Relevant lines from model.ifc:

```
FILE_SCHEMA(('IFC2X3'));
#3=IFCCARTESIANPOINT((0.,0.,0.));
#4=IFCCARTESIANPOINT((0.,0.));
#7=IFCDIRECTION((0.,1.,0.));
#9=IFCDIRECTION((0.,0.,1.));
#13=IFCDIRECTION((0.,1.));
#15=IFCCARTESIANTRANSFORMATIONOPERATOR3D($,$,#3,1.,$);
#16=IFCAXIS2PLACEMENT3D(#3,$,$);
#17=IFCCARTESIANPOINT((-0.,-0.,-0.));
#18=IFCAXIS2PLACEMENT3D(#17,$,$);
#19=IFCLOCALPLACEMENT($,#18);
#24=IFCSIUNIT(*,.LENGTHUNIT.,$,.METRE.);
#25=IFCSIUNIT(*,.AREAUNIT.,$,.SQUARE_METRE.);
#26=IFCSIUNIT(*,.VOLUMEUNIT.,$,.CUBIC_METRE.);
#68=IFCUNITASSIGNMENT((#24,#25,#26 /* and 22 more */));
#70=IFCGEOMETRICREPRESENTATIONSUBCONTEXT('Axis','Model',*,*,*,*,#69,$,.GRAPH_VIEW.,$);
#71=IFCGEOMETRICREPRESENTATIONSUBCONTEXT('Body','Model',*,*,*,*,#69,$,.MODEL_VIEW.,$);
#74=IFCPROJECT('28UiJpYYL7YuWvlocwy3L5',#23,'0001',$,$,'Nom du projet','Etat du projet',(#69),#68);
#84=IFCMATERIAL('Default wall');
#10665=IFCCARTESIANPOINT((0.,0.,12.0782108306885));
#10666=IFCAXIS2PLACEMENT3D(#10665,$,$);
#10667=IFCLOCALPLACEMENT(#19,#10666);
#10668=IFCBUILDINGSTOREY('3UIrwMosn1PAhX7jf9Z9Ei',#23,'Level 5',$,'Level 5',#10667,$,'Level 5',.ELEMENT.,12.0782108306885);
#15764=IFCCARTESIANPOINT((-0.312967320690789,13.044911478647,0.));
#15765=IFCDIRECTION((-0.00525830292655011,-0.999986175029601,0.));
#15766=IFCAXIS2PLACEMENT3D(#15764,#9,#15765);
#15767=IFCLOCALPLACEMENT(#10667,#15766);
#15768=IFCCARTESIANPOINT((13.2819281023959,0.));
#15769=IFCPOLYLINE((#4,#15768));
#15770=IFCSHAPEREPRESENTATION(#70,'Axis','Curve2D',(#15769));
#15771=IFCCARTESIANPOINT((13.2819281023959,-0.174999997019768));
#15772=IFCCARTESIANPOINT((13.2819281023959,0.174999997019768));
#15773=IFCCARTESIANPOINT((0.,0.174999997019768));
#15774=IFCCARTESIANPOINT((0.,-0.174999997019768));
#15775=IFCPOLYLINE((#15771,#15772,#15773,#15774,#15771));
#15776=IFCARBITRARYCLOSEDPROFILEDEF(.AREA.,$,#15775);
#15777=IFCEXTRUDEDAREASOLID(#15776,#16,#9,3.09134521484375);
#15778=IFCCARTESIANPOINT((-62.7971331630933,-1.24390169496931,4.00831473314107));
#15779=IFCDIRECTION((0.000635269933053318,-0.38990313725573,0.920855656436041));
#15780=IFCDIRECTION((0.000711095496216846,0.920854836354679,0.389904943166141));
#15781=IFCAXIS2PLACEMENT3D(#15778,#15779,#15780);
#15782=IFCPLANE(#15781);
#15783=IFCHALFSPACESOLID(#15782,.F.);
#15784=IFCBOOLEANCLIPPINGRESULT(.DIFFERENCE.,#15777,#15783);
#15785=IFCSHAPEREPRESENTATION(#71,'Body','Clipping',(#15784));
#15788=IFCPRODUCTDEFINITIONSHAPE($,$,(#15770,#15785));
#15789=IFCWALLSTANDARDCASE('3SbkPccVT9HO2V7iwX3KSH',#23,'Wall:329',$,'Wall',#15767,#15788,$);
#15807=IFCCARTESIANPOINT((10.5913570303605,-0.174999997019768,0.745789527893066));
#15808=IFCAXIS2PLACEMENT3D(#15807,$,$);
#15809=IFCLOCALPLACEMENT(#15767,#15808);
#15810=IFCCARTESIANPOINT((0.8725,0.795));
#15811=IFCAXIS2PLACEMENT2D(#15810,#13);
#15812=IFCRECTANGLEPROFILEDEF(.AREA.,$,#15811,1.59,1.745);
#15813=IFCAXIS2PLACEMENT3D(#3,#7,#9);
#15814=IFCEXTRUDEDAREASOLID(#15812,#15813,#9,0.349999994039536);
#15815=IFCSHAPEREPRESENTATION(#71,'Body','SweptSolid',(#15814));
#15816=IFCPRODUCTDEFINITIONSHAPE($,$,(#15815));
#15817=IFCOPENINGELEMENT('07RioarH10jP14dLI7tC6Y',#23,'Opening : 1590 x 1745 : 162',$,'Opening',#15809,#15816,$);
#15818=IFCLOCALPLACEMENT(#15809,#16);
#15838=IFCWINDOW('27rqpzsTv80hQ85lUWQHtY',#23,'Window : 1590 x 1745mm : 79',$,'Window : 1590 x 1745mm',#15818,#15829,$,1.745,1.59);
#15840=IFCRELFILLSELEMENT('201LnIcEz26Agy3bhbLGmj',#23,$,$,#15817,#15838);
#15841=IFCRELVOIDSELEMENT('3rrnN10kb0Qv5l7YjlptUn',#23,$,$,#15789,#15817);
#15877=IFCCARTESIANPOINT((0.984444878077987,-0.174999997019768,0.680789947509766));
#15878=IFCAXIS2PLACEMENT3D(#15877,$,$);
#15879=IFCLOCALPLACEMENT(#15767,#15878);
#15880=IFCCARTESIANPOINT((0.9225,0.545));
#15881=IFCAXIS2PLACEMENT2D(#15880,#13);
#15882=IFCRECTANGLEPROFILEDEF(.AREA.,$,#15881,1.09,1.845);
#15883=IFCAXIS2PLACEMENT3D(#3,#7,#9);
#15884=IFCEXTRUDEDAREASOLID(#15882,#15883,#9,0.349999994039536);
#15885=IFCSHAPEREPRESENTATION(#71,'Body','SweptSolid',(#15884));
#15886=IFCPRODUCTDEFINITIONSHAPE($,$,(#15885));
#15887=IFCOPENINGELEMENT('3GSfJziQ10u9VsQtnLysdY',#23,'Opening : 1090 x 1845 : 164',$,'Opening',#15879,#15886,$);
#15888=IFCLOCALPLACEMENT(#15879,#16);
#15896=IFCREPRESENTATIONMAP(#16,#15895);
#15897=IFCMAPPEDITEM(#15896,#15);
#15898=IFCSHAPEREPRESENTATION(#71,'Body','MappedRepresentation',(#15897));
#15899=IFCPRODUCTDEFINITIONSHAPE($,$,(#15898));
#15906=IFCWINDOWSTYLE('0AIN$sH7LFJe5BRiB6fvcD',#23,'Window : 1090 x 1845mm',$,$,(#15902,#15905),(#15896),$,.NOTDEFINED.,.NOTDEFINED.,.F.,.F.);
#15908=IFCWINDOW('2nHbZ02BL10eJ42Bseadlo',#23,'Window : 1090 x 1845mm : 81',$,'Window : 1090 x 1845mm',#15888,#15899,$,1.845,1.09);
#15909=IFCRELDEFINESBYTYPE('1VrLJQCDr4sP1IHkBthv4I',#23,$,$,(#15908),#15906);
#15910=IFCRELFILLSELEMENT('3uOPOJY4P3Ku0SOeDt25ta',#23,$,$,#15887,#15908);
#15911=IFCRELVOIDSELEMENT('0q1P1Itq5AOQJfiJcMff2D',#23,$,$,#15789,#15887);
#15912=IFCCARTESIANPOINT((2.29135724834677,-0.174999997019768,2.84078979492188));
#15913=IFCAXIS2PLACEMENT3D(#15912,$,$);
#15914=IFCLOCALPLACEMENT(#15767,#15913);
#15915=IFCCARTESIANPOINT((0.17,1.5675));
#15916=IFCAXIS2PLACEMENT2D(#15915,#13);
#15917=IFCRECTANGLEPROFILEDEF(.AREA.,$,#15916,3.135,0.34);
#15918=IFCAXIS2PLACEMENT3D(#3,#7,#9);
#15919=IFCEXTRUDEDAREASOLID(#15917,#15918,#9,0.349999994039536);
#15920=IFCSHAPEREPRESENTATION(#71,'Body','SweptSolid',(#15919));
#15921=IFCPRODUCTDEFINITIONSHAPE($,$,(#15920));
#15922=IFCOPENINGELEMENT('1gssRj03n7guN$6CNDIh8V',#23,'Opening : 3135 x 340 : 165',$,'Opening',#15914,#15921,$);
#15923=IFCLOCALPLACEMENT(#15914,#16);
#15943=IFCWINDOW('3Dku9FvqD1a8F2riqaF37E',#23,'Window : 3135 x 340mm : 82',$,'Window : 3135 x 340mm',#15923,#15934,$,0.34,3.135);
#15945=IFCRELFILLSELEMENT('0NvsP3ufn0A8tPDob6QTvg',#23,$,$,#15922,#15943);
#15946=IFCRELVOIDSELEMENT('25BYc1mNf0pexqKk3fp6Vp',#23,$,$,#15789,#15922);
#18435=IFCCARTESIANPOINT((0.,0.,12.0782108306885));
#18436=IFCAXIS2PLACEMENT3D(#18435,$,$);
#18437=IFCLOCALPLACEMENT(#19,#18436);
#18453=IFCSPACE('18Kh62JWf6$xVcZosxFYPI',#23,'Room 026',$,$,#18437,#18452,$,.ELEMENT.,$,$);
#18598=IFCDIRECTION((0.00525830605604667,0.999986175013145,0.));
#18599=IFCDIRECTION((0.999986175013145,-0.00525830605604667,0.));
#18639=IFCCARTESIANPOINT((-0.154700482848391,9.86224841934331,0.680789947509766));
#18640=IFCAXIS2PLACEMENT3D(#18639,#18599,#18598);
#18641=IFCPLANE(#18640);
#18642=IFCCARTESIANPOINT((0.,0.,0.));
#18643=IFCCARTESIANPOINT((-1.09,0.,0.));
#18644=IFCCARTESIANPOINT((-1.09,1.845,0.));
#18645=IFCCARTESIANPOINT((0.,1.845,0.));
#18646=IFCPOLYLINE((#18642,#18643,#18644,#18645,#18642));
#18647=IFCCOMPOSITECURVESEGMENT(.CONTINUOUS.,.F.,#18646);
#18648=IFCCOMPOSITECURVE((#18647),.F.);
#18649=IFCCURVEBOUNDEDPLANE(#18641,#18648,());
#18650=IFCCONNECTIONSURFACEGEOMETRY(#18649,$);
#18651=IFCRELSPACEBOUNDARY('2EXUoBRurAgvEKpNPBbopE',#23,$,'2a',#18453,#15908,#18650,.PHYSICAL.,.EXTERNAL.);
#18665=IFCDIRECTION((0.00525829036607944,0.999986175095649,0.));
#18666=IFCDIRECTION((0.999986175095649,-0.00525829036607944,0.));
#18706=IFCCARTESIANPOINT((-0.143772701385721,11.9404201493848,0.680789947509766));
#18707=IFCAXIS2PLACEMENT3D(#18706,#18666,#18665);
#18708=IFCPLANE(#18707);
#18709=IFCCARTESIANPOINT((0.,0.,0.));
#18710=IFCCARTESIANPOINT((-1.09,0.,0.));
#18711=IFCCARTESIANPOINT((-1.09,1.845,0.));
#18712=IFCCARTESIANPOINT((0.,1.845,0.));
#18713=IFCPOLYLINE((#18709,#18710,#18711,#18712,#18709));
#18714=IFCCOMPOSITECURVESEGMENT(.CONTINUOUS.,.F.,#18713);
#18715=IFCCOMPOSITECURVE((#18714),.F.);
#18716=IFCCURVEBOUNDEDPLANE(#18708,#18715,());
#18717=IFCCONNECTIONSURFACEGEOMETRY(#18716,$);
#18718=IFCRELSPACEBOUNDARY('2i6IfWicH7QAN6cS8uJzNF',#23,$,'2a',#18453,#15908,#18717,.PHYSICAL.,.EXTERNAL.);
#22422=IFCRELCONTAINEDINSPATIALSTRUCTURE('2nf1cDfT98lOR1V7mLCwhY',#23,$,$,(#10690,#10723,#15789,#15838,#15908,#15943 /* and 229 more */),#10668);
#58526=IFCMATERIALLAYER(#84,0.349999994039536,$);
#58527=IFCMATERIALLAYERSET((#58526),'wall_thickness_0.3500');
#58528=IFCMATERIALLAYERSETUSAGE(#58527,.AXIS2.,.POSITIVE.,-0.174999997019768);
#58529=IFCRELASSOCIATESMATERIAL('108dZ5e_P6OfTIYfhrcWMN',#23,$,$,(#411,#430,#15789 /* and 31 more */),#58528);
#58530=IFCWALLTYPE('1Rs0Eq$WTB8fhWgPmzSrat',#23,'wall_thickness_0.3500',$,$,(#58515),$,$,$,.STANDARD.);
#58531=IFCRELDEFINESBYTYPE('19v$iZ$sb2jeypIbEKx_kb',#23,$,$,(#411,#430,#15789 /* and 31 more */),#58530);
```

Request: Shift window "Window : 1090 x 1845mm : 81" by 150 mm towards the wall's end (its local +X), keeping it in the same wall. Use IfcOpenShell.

```python
import numpy as np
import ifcopenshell
import ifcopenshell.api.geometry
import ifcopenshell.util.placement

model = ifcopenshell.open("model.ifc")

window = model.by_id(15908)
opening = window.FillsVoids[0].RelatingOpeningElement
wall = opening.VoidsElements[0].RelatingBuildingElement

wall_matrix = ifcopenshell.util.placement.get_local_placement(wall.ObjectPlacement)
shift = wall_matrix[:3, 0] * 0.15
before = ifcopenshell.util.placement.get_local_placement(window.ObjectPlacement)[:3, 3].copy()

# The window is placed relative to its opening, so it follows when the opening moves.
matrix = ifcopenshell.util.placement.get_local_placement(opening.ObjectPlacement)
matrix[:3, 3] += shift
ifcopenshell.api.geometry.edit_object_placement(
    model, product=opening, matrix=matrix, is_si=False, should_transform_children=True
)

# Space boundary surfaces are stored in each space's coordinates; move them too.
for rel in window.ProvidesBoundaries:
    if not rel.ConnectionGeometry:
        continue
    surface = rel.ConnectionGeometry.SurfaceOnRelatingElement.BasisSurface
    space_matrix = ifcopenshell.util.placement.get_local_placement(rel.RelatingSpace.ObjectPlacement)
    point = np.array(surface.Position.Location.Coordinates) + space_matrix[:3, :3].T @ shift
    surface.Position = model.createIfcAxis2Placement3D(
        model.createIfcCartesianPoint(point.tolist()), surface.Position.Axis, surface.Position.RefDirection
    )

after = ifcopenshell.util.placement.get_local_placement(window.ObjectPlacement)[:3, 3]
print("window moved by", (after - before).round(3) + 0.0)

model.write("model_rev.ifc")
```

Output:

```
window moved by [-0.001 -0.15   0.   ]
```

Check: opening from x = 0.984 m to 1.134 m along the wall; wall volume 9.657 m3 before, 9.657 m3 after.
